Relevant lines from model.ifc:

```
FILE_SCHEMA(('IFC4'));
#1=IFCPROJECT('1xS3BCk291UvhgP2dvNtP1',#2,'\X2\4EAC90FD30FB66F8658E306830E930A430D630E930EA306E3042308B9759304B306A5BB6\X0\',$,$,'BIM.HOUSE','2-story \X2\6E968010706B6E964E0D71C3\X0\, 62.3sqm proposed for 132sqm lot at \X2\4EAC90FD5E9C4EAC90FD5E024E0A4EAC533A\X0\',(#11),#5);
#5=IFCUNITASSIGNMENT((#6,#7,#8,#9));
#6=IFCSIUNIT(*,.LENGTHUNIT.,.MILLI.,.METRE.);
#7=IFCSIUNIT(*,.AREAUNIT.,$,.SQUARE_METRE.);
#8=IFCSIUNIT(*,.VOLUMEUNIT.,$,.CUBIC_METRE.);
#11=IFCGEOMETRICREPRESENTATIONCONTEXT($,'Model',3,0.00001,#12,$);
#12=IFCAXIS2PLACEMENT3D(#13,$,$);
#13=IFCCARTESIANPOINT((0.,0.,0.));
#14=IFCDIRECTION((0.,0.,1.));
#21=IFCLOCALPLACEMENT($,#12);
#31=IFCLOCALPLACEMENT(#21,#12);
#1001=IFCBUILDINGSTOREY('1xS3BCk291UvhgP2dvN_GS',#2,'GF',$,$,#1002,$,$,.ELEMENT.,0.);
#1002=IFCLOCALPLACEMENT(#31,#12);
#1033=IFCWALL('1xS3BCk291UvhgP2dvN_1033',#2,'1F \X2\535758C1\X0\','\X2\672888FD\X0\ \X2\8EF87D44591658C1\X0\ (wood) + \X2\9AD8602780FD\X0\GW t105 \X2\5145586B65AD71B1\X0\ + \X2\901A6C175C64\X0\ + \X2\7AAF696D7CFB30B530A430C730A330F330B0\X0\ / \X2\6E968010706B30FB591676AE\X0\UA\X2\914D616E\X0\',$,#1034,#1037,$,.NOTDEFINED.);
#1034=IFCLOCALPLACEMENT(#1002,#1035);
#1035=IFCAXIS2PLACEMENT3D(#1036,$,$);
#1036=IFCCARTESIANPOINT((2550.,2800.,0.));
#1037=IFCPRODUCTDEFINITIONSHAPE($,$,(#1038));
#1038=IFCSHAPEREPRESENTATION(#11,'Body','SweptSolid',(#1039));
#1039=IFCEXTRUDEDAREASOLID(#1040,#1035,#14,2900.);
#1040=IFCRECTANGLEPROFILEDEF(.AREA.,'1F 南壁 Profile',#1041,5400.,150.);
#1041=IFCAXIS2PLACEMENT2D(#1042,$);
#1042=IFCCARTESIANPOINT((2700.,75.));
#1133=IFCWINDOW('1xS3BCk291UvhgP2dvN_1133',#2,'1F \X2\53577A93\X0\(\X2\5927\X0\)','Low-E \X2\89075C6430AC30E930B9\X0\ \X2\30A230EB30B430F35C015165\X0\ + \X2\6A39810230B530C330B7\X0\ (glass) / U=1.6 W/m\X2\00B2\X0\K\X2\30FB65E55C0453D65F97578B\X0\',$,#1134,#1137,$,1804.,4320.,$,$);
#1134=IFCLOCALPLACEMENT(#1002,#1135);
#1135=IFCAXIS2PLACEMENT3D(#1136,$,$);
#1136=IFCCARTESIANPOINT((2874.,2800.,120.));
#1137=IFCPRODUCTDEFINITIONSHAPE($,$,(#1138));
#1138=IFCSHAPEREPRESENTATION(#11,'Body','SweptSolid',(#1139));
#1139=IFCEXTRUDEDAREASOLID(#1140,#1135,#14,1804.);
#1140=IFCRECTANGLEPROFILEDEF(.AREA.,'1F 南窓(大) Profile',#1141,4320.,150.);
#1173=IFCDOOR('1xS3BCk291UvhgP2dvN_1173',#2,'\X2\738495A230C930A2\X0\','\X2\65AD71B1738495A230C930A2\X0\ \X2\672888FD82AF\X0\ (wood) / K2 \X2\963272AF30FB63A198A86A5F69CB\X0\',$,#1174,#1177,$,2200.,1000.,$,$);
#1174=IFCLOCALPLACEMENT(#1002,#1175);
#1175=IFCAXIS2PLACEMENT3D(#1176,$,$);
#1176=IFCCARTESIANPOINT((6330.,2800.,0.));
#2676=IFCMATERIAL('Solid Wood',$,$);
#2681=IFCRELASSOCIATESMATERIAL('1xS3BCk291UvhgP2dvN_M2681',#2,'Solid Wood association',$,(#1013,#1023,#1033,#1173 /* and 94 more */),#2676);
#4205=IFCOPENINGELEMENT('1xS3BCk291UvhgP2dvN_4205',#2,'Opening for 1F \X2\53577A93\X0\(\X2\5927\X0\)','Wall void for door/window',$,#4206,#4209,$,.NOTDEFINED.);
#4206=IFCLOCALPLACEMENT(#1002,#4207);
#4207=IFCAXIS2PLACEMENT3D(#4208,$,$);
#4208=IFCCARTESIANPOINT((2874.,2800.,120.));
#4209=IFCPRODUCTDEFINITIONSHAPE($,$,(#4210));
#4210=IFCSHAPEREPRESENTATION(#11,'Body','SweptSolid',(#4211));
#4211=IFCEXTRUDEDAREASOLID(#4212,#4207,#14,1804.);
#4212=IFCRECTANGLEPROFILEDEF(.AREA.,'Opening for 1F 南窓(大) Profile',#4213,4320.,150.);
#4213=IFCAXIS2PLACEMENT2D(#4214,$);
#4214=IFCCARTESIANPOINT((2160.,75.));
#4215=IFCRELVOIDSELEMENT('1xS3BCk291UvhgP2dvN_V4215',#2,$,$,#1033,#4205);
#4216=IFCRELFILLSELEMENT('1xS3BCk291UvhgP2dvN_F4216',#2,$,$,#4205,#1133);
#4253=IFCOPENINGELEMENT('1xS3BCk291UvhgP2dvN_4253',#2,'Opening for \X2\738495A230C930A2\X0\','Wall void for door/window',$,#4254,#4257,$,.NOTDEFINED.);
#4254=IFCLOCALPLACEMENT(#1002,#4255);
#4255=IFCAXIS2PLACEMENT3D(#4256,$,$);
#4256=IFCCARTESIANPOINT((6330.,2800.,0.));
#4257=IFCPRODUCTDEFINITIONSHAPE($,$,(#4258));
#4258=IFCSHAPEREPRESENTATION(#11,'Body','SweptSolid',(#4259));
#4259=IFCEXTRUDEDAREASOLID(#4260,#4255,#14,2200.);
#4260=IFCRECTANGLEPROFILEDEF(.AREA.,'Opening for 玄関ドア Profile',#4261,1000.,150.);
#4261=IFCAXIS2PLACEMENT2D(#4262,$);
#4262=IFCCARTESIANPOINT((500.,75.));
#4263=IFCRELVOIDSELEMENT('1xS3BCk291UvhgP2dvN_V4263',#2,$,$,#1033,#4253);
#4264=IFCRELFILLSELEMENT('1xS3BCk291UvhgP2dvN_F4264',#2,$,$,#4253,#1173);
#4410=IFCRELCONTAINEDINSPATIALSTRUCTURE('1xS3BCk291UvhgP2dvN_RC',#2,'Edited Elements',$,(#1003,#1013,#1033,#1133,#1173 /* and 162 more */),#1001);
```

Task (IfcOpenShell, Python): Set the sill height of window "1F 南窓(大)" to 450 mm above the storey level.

```python
import numpy as np
import ifcopenshell
import ifcopenshell.api.geometry
import ifcopenshell.geom
import ifcopenshell.util.element
import ifcopenshell.util.placement
import ifcopenshell.util.shape
import ifcopenshell.util.unit

model = ifcopenshell.open("model.ifc")
unit_scale = ifcopenshell.util.unit.calculate_unit_scale(model)

window = model.by_id(1133)
opening = window.FillsVoids[0].RelatingOpeningElement
storey = ifcopenshell.util.element.get_container(window, ifc_class="IfcBuildingStorey")
level = ifcopenshell.util.placement.get_local_placement(storey.ObjectPlacement)[2, 3]

# The opening's origin need not be at the sill, so measure its lowest point.
shape = ifcopenshell.geom.create_shape(ifcopenshell.geom.settings(), opening)
bottom = ifcopenshell.util.shape.get_shape_bottom_elevation(shape, shape.geometry) / unit_scale
dz = level + 0.45 / unit_scale - bottom

shift = np.array([0.0, 0.0, dz])
# The window is not placed relative to its opening, so move both.
for product in (opening, window):
    matrix = ifcopenshell.util.placement.get_local_placement(product.ObjectPlacement)
    matrix[:3, 3] += shift
    ifcopenshell.api.geometry.edit_object_placement(model, product=product, matrix=matrix, is_si=False)

print(f"moved by {dz * unit_scale:+.3f} m")

model.write("model_rev.ifc")
```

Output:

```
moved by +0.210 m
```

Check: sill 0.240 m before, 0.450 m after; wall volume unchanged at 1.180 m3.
